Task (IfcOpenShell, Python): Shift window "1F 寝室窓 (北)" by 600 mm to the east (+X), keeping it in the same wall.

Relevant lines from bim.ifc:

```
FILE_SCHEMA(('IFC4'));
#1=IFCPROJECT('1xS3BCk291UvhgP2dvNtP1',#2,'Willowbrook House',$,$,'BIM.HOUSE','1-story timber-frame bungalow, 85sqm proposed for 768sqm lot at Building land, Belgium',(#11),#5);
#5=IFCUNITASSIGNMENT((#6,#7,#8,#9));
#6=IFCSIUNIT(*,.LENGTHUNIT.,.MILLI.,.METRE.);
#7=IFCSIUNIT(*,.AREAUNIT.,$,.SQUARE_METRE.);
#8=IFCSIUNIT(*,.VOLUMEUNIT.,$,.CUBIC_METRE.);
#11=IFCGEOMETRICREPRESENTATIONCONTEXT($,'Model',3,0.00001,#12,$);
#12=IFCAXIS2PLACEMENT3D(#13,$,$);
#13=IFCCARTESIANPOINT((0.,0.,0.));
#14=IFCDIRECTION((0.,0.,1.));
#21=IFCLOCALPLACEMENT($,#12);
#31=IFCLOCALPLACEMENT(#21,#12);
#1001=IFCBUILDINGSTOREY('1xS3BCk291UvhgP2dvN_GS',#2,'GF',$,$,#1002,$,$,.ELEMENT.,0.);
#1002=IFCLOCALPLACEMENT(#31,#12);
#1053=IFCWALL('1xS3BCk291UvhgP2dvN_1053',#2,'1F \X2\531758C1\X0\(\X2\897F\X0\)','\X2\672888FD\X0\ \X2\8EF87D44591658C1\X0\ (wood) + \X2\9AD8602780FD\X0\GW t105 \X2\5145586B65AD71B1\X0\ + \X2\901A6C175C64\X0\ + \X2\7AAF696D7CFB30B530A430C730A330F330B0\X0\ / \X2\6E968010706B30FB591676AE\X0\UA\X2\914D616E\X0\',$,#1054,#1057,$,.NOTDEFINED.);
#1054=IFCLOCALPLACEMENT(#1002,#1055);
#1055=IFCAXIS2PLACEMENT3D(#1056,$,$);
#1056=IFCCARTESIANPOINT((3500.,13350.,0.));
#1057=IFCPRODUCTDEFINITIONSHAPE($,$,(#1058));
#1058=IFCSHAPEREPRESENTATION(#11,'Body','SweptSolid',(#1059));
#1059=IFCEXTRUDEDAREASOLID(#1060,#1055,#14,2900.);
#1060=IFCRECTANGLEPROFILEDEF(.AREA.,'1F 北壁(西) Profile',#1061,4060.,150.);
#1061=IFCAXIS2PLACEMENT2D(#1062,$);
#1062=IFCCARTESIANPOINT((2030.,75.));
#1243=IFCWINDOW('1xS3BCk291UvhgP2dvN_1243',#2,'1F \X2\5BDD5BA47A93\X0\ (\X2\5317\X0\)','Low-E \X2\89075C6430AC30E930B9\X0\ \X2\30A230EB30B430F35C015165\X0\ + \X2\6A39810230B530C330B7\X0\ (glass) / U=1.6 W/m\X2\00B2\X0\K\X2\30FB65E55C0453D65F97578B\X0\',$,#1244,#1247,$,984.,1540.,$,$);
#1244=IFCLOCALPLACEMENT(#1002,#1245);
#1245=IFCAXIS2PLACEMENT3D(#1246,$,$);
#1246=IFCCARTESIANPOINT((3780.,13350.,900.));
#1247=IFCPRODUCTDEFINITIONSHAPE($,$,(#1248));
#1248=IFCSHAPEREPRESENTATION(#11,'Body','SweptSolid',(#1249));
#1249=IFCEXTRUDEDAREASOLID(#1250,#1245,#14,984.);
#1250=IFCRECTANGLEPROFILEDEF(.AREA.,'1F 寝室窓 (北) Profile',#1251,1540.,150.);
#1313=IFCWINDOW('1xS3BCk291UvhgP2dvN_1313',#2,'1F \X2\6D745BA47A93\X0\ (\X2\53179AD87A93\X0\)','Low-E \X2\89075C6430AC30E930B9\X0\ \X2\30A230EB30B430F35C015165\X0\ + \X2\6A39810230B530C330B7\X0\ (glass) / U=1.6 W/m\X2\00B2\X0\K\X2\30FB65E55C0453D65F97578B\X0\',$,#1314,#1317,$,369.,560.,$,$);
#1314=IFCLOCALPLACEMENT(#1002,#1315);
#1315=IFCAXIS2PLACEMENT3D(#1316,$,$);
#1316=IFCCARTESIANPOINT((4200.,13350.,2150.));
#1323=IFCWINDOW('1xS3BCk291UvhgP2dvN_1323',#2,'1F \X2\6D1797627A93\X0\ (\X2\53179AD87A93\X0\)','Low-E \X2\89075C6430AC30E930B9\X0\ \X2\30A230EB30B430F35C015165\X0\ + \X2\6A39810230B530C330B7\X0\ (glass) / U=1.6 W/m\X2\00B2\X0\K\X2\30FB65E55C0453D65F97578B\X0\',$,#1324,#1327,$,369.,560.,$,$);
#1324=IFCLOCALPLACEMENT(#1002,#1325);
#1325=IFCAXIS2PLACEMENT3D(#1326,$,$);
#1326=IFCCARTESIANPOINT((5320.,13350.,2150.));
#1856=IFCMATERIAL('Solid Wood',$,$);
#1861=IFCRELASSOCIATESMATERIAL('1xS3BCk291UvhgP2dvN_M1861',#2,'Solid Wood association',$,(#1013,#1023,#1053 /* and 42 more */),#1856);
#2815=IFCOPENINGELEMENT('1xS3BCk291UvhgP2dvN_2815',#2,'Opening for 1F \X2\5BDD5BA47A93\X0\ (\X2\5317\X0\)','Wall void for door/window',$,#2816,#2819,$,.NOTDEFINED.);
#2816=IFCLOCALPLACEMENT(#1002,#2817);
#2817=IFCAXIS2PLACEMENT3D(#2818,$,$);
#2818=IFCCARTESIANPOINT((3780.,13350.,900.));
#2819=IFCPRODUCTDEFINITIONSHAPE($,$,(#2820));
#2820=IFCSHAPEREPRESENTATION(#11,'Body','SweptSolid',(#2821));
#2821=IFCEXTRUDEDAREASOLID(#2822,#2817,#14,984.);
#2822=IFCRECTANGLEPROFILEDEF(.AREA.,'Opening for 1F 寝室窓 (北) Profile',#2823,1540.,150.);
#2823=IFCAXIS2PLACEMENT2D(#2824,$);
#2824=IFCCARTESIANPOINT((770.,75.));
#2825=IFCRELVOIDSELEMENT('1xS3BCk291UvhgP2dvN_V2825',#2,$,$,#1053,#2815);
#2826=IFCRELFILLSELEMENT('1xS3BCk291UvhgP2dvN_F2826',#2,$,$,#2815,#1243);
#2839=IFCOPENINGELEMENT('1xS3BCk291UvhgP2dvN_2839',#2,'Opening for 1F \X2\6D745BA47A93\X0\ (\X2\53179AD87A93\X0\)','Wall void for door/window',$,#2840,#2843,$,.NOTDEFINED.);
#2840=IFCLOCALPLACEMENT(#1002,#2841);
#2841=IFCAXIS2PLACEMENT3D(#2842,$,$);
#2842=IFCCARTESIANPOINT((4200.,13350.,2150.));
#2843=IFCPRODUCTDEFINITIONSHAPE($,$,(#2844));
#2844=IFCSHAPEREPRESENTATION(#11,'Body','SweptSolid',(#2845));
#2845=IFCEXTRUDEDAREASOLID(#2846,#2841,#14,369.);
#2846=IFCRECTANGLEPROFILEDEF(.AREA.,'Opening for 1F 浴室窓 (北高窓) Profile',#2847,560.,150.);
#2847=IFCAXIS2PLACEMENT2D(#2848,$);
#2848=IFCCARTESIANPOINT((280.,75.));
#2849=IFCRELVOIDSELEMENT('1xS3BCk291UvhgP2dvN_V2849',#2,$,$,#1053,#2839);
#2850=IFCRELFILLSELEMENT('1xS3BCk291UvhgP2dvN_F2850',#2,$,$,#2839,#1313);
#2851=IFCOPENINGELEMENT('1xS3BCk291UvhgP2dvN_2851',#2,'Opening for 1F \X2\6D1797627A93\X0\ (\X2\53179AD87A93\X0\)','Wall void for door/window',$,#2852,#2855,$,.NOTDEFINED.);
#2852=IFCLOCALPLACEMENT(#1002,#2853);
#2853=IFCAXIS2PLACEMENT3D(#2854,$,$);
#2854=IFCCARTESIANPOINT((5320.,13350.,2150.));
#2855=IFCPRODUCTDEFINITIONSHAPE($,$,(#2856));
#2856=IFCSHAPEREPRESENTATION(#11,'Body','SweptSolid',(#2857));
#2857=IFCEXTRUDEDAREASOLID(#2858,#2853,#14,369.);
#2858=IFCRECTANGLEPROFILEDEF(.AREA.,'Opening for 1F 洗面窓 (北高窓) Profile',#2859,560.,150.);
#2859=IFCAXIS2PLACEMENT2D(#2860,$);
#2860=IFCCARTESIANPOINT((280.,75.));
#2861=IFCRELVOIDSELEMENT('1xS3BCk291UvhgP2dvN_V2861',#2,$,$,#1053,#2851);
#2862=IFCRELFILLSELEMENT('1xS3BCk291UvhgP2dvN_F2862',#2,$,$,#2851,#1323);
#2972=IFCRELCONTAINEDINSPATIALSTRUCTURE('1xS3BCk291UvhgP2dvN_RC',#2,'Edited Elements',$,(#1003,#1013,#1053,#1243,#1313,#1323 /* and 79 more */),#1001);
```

```python
import ifcopenshell
import ifcopenshell.api.geometry
import ifcopenshell.util.placement
import ifcopenshell.util.unit

model = ifcopenshell.open("bim.ifc")
unit_scale = ifcopenshell.util.unit.calculate_unit_scale(model)

window = model.by_guid("1xS3BCk291UvhgP2dvN_1243")
opening = window.FillsVoids[0].RelatingOpeningElement
wall = opening.VoidsElements[0].RelatingBuildingElement

wall_matrix = ifcopenshell.util.placement.get_local_placement(wall.ObjectPlacement)
shift = wall_matrix[:3, 0] * 0.6 / unit_scale
before = ifcopenshell.util.placement.get_local_placement(window.ObjectPlacement)[:3, 3].copy()

# The window is not placed relative to its opening, so move both.
for product in (opening, window):
    matrix = ifcopenshell.util.placement.get_local_placement(product.ObjectPlacement)
    matrix[:3, 3] += shift
    ifcopenshell.api.geometry.edit_object_placement(model, product=product, matrix=matrix, is_si=False)

after = ifcopenshell.util.placement.get_local_placement(window.ObjectPlacement)[:3, 3]
print("window moved by", (after - before).round(3) + 0.0)

model.write("bim_updated.ifc")
```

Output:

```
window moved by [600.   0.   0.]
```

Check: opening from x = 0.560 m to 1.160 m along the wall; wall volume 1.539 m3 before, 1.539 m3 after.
